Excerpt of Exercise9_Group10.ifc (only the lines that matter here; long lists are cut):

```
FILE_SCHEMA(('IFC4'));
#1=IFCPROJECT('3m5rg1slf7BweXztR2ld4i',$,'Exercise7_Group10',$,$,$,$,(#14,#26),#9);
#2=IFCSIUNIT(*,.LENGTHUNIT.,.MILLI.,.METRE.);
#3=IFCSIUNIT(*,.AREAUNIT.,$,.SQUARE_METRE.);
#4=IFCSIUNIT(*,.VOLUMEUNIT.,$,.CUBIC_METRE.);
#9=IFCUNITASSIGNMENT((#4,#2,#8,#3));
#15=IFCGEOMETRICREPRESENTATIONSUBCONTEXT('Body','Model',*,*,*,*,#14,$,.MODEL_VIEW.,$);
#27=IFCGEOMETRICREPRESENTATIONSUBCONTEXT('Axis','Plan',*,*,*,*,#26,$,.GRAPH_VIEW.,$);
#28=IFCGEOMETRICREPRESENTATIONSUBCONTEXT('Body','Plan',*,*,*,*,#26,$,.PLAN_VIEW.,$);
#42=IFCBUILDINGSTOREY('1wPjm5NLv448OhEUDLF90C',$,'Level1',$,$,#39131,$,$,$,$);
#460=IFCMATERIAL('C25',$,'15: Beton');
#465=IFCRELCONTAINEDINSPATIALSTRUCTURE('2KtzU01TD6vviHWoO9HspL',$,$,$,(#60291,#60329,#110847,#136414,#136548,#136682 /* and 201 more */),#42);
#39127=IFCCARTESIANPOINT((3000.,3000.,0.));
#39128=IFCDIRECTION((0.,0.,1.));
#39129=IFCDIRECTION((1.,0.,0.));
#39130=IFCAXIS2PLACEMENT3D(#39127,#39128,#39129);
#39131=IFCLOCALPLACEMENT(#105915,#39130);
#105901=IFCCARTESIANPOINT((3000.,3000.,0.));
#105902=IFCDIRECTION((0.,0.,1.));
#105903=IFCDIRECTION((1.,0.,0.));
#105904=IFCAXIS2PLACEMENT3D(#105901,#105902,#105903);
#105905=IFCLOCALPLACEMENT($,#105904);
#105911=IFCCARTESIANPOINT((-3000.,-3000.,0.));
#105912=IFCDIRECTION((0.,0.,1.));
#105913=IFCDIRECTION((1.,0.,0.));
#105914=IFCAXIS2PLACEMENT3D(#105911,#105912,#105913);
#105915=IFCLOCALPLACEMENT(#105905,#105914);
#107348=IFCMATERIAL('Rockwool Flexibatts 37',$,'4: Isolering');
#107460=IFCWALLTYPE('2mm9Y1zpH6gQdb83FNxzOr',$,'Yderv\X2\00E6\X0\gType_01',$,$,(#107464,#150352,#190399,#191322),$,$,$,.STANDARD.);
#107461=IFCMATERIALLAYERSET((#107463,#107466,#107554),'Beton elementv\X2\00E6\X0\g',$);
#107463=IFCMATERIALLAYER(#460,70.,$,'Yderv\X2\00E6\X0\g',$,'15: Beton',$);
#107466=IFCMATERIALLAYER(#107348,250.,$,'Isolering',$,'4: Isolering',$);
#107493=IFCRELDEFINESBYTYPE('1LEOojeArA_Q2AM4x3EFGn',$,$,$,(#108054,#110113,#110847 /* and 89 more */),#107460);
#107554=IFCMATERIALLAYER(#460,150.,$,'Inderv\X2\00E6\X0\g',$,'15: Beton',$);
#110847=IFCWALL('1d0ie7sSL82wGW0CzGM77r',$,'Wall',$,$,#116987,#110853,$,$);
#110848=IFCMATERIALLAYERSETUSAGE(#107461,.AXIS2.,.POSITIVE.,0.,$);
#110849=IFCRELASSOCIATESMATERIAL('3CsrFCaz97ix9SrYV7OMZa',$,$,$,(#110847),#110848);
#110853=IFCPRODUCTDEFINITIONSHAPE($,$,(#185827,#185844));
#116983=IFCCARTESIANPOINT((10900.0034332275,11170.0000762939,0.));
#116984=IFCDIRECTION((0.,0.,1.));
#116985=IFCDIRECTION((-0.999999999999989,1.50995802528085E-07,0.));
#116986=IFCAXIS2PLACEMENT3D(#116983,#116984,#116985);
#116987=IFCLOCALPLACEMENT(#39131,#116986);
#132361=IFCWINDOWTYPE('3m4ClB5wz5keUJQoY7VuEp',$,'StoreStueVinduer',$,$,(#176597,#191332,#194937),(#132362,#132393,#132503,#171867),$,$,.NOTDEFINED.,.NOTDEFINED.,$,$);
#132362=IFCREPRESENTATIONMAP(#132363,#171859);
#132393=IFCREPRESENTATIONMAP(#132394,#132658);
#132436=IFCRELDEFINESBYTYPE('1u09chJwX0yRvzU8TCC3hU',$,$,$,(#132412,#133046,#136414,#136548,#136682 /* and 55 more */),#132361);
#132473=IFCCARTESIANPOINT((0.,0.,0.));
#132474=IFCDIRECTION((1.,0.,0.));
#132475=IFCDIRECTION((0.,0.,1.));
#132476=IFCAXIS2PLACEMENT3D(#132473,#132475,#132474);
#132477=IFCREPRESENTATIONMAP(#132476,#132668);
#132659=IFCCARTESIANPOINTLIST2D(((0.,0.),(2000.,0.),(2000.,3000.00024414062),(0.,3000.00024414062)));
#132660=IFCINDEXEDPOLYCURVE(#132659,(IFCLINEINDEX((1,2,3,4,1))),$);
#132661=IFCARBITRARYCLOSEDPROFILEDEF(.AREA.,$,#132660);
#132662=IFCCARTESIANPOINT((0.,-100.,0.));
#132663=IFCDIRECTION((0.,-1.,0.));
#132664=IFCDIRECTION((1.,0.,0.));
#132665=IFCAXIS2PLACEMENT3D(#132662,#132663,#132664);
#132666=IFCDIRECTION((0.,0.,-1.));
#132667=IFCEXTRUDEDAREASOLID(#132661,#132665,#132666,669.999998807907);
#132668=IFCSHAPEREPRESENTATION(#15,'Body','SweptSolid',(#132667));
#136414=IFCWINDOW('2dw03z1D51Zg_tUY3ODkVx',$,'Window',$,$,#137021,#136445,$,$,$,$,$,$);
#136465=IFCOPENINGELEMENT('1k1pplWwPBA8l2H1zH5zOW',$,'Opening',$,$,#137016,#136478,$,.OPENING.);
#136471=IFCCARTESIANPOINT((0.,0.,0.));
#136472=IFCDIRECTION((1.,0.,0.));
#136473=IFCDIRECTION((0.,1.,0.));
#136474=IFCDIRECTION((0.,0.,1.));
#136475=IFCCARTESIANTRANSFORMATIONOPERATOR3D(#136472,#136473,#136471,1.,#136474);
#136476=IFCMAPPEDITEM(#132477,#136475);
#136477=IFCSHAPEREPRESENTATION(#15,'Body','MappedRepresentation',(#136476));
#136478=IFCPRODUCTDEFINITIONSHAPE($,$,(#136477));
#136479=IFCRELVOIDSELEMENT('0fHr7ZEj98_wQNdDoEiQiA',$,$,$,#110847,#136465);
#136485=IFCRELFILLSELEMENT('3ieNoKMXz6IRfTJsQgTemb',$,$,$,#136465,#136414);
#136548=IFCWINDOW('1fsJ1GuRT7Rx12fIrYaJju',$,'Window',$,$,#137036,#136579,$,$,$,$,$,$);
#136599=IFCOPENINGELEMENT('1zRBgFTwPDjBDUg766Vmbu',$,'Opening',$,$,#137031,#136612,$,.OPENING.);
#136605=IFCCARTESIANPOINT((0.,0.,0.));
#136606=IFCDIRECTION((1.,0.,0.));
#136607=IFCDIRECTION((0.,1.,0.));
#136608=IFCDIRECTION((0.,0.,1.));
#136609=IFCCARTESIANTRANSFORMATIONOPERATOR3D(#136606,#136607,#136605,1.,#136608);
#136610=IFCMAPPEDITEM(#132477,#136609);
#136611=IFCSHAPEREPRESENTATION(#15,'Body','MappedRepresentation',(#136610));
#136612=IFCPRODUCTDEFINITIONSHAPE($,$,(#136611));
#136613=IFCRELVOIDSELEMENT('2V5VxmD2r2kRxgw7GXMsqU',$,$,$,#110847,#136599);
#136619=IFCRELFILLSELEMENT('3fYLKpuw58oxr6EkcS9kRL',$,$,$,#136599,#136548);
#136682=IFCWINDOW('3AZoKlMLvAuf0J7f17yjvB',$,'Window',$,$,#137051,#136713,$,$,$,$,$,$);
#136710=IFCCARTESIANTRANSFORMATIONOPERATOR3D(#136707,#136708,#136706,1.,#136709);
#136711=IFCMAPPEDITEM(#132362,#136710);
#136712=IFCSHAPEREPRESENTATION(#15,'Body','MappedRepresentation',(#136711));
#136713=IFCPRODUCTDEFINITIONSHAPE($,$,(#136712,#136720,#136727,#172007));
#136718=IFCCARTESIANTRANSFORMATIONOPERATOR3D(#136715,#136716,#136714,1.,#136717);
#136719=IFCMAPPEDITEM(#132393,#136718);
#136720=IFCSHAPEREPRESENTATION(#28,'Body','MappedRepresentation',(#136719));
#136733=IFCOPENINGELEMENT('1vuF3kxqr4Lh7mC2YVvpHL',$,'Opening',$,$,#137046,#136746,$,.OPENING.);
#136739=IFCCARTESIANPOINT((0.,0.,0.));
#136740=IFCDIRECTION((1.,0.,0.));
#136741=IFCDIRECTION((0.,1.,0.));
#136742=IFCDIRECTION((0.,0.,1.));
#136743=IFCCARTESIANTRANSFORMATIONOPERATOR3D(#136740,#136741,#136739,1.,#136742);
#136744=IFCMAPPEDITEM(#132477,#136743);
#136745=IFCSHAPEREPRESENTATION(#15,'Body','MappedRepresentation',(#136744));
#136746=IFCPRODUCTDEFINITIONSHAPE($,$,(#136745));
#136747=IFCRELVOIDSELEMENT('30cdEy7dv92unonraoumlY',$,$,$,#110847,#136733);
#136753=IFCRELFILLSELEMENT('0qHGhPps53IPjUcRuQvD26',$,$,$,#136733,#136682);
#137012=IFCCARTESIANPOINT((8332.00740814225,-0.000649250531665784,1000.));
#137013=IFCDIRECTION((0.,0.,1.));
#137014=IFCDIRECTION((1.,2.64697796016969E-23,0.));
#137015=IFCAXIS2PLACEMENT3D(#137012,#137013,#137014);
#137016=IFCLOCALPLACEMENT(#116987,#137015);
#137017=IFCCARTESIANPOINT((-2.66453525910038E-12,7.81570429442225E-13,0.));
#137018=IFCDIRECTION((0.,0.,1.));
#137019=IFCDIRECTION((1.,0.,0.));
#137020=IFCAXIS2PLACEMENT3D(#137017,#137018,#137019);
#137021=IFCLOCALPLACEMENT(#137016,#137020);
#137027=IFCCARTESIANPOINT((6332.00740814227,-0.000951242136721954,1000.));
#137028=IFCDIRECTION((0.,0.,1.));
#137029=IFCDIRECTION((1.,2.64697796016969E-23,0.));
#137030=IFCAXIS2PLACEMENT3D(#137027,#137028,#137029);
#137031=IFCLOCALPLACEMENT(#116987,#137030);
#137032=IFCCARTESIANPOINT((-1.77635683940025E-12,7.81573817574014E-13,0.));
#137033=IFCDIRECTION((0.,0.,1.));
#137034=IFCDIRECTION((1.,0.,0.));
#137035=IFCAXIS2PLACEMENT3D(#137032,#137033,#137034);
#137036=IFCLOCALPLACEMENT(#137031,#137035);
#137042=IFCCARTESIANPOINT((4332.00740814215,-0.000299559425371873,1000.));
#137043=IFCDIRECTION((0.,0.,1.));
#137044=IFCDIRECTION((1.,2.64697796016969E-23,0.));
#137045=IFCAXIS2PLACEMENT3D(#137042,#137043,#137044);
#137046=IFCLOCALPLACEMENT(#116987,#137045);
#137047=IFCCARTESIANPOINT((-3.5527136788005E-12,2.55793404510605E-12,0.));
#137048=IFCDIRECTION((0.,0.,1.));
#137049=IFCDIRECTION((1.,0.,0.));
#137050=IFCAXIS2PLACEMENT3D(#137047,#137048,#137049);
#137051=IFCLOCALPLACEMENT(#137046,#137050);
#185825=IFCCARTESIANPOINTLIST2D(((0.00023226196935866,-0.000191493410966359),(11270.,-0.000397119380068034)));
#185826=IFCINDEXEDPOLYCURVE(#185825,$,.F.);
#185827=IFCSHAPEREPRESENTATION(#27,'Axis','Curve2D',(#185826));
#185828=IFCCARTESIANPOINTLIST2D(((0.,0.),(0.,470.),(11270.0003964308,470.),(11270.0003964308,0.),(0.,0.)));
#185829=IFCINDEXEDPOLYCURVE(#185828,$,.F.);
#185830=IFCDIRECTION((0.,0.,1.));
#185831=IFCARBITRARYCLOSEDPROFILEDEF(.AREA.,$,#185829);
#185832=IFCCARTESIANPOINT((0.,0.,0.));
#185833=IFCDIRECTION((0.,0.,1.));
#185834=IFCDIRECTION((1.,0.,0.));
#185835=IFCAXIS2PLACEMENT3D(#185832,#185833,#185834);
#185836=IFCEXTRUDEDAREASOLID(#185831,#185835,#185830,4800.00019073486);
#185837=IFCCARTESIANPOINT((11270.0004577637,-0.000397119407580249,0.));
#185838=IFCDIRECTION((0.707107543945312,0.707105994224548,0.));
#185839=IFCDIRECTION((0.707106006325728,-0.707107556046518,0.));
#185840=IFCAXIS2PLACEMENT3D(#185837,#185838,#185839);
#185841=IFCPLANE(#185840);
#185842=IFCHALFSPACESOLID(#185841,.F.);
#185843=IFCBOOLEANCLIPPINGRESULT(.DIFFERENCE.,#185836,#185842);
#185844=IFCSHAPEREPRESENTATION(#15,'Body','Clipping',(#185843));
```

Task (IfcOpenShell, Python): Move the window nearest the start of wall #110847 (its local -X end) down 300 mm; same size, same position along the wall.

```python
import numpy as np
import ifcopenshell
import ifcopenshell.api.geometry
import ifcopenshell.util.placement
import ifcopenshell.util.unit

model = ifcopenshell.open("Exercise9_Group10.ifc")
unit_scale = ifcopenshell.util.unit.calculate_unit_scale(model)

window = model.by_guid("3AZoKlMLvAuf0J7f17yjvB")
opening = window.FillsVoids[0].RelatingOpeningElement
dz = -300.0

shift = np.array([0.0, 0.0, dz])
# The window is placed relative to its opening, so it follows when the opening moves.
matrix = ifcopenshell.util.placement.get_local_placement(opening.ObjectPlacement)
matrix[:3, 3] += shift
ifcopenshell.api.geometry.edit_object_placement(
    model, product=opening, matrix=matrix, is_si=False, should_transform_children=True
)

print(f"moved by {dz * unit_scale:+.3f} m")

model.write("Exercise9_Group10_rev.ifc")
```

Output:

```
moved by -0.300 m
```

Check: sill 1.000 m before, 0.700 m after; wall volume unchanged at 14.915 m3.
